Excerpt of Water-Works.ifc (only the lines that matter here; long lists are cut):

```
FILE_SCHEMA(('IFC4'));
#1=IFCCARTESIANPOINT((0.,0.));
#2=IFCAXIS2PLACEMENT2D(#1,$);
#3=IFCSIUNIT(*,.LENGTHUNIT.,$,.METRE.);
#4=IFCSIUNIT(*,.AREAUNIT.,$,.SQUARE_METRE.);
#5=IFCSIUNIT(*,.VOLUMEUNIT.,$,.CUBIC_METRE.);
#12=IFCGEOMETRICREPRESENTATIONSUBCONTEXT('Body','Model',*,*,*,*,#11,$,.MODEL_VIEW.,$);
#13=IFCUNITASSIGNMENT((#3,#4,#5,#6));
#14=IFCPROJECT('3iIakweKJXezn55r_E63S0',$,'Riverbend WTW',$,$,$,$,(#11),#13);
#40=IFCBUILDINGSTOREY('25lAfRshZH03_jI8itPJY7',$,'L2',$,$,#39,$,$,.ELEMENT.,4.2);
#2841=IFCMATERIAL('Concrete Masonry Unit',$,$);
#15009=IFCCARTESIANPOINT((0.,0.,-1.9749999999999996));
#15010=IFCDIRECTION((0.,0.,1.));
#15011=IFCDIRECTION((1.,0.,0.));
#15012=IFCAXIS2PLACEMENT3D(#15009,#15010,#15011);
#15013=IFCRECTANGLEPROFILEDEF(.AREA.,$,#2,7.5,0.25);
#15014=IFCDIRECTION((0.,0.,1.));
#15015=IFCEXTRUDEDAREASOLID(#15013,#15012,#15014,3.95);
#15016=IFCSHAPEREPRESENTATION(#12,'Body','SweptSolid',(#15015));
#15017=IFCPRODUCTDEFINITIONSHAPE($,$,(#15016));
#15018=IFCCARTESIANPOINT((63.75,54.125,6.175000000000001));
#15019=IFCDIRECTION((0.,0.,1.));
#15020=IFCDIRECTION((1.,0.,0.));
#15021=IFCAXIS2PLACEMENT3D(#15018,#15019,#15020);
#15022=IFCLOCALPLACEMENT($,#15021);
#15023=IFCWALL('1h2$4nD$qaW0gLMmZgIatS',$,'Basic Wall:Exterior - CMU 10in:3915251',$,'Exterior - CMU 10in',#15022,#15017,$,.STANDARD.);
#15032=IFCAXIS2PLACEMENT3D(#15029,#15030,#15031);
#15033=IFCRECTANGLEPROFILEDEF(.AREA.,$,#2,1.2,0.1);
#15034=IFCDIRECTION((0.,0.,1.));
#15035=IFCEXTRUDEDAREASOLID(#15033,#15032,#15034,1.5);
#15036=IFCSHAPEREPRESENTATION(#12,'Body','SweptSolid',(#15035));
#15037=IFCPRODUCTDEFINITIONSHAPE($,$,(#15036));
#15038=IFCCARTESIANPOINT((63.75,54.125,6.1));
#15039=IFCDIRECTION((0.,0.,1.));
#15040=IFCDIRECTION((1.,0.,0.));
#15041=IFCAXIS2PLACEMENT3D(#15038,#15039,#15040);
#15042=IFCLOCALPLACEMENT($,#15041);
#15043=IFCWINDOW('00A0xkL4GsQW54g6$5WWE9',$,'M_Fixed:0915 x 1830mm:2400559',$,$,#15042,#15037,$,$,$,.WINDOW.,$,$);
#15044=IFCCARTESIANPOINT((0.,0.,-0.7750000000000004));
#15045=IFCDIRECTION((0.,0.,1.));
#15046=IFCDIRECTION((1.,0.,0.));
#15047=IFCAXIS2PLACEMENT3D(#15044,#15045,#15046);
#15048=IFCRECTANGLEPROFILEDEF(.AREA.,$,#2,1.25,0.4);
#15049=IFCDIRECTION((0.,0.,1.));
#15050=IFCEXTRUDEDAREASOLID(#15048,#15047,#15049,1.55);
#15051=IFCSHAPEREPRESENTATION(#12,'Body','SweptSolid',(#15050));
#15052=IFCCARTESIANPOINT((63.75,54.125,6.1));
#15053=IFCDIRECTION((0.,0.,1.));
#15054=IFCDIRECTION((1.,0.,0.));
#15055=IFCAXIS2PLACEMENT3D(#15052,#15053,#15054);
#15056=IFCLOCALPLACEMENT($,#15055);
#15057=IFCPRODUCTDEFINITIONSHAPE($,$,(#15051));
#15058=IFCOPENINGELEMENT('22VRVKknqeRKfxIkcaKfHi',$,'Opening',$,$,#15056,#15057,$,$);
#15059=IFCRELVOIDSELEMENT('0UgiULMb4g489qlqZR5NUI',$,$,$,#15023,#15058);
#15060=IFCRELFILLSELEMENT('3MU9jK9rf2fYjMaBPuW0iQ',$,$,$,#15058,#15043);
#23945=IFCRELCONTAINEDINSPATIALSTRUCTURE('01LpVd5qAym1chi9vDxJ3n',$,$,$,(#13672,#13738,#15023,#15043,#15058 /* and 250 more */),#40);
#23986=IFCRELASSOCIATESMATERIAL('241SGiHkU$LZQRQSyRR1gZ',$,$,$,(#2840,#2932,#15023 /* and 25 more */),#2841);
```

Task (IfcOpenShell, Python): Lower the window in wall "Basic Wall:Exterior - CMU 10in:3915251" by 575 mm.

```python
import numpy as np
import ifcopenshell
import ifcopenshell.api.geometry
import ifcopenshell.util.placement
import ifcopenshell.util.unit

model = ifcopenshell.open("Water-Works.ifc")
unit_scale = ifcopenshell.util.unit.calculate_unit_scale(model)

window = model.by_id(15043)
opening = window.FillsVoids[0].RelatingOpeningElement
dz = -0.575 / unit_scale

shift = np.array([0.0, 0.0, dz])
# The window is not placed relative to its opening, so move both.
for product in (opening, window):
    matrix = ifcopenshell.util.placement.get_local_placement(product.ObjectPlacement)
    matrix[:3, 3] += shift
    ifcopenshell.api.geometry.edit_object_placement(model, product=product, matrix=matrix, is_si=False)

print(f"moved by {dz * unit_scale:+.3f} m")

model.write("Water-Works_rev.ifc")
```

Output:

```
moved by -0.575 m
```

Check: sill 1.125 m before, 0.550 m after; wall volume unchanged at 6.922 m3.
